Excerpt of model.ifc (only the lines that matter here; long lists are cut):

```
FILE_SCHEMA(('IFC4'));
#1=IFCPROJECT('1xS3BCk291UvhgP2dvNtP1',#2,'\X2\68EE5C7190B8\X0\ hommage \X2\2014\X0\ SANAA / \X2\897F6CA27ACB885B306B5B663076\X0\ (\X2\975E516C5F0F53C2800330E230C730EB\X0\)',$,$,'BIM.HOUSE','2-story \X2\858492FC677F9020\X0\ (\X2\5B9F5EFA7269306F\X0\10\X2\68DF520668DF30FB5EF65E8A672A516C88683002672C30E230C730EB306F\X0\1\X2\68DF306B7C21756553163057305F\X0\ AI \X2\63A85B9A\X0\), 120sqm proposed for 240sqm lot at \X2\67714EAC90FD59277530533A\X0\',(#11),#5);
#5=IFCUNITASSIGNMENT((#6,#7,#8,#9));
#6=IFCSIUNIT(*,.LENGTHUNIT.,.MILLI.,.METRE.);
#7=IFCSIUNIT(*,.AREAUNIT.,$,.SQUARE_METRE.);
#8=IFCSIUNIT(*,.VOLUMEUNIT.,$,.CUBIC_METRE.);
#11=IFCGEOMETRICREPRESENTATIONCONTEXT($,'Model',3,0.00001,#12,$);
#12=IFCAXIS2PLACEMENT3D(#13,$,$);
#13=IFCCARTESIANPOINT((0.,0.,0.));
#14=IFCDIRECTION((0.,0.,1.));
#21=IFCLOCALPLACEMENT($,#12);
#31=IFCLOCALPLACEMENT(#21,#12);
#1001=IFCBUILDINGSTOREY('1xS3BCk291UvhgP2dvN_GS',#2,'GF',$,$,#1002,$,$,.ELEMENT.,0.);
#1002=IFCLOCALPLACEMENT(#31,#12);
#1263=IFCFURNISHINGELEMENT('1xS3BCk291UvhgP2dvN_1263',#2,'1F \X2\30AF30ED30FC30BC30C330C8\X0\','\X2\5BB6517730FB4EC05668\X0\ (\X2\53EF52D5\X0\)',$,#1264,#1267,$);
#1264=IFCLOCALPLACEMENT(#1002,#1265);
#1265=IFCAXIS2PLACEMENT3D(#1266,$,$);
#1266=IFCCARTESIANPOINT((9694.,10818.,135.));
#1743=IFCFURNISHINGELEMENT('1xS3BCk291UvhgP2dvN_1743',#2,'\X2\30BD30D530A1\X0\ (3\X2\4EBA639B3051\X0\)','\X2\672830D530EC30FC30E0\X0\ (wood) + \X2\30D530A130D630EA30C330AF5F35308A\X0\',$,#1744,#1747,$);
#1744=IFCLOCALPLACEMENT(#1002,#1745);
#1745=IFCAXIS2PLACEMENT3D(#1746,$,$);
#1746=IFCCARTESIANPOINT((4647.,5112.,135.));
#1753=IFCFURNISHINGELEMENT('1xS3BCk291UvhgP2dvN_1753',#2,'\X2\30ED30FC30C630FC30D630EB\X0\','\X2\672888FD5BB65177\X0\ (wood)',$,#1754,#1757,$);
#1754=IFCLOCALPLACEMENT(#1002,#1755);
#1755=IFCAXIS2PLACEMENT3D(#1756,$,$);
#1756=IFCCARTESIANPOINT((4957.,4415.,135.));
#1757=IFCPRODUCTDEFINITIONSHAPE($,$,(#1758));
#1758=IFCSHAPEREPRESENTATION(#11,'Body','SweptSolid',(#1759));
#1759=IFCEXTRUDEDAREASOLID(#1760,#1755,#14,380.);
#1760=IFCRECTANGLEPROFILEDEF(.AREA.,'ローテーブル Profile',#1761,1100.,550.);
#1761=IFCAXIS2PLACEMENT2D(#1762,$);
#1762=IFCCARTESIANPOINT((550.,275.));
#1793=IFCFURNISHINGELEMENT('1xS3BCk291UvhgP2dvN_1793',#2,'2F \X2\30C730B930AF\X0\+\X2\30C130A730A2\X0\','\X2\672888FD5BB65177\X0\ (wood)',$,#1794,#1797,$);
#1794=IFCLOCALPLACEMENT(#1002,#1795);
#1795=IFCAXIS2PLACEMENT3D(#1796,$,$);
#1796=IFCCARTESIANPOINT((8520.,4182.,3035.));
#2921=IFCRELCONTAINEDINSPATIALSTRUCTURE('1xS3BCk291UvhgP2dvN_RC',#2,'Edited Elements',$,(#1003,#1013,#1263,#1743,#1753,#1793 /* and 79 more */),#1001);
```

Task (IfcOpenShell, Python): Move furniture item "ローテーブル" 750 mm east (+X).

```python
import ifcopenshell
import ifcopenshell.api.geometry
import ifcopenshell.util.placement
import ifcopenshell.util.unit

model = ifcopenshell.open("model.ifc")
unit_scale = ifcopenshell.util.unit.calculate_unit_scale(model)

item = model.by_guid("1xS3BCk291UvhgP2dvN_1753")
matrix = ifcopenshell.util.placement.get_local_placement(item.ObjectPlacement)
matrix[0, 3] += 0.75 / unit_scale
ifcopenshell.api.geometry.edit_object_placement(model, product=item, matrix=matrix, is_si=False)

print(ifcopenshell.util.placement.get_local_placement(item.ObjectPlacement).round(3) + 0.0)

model.write("model_rev.ifc")
```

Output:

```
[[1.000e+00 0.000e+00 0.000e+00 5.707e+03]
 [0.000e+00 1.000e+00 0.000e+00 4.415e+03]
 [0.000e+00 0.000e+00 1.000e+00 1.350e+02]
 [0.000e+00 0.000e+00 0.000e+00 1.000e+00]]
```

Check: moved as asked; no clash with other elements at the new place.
